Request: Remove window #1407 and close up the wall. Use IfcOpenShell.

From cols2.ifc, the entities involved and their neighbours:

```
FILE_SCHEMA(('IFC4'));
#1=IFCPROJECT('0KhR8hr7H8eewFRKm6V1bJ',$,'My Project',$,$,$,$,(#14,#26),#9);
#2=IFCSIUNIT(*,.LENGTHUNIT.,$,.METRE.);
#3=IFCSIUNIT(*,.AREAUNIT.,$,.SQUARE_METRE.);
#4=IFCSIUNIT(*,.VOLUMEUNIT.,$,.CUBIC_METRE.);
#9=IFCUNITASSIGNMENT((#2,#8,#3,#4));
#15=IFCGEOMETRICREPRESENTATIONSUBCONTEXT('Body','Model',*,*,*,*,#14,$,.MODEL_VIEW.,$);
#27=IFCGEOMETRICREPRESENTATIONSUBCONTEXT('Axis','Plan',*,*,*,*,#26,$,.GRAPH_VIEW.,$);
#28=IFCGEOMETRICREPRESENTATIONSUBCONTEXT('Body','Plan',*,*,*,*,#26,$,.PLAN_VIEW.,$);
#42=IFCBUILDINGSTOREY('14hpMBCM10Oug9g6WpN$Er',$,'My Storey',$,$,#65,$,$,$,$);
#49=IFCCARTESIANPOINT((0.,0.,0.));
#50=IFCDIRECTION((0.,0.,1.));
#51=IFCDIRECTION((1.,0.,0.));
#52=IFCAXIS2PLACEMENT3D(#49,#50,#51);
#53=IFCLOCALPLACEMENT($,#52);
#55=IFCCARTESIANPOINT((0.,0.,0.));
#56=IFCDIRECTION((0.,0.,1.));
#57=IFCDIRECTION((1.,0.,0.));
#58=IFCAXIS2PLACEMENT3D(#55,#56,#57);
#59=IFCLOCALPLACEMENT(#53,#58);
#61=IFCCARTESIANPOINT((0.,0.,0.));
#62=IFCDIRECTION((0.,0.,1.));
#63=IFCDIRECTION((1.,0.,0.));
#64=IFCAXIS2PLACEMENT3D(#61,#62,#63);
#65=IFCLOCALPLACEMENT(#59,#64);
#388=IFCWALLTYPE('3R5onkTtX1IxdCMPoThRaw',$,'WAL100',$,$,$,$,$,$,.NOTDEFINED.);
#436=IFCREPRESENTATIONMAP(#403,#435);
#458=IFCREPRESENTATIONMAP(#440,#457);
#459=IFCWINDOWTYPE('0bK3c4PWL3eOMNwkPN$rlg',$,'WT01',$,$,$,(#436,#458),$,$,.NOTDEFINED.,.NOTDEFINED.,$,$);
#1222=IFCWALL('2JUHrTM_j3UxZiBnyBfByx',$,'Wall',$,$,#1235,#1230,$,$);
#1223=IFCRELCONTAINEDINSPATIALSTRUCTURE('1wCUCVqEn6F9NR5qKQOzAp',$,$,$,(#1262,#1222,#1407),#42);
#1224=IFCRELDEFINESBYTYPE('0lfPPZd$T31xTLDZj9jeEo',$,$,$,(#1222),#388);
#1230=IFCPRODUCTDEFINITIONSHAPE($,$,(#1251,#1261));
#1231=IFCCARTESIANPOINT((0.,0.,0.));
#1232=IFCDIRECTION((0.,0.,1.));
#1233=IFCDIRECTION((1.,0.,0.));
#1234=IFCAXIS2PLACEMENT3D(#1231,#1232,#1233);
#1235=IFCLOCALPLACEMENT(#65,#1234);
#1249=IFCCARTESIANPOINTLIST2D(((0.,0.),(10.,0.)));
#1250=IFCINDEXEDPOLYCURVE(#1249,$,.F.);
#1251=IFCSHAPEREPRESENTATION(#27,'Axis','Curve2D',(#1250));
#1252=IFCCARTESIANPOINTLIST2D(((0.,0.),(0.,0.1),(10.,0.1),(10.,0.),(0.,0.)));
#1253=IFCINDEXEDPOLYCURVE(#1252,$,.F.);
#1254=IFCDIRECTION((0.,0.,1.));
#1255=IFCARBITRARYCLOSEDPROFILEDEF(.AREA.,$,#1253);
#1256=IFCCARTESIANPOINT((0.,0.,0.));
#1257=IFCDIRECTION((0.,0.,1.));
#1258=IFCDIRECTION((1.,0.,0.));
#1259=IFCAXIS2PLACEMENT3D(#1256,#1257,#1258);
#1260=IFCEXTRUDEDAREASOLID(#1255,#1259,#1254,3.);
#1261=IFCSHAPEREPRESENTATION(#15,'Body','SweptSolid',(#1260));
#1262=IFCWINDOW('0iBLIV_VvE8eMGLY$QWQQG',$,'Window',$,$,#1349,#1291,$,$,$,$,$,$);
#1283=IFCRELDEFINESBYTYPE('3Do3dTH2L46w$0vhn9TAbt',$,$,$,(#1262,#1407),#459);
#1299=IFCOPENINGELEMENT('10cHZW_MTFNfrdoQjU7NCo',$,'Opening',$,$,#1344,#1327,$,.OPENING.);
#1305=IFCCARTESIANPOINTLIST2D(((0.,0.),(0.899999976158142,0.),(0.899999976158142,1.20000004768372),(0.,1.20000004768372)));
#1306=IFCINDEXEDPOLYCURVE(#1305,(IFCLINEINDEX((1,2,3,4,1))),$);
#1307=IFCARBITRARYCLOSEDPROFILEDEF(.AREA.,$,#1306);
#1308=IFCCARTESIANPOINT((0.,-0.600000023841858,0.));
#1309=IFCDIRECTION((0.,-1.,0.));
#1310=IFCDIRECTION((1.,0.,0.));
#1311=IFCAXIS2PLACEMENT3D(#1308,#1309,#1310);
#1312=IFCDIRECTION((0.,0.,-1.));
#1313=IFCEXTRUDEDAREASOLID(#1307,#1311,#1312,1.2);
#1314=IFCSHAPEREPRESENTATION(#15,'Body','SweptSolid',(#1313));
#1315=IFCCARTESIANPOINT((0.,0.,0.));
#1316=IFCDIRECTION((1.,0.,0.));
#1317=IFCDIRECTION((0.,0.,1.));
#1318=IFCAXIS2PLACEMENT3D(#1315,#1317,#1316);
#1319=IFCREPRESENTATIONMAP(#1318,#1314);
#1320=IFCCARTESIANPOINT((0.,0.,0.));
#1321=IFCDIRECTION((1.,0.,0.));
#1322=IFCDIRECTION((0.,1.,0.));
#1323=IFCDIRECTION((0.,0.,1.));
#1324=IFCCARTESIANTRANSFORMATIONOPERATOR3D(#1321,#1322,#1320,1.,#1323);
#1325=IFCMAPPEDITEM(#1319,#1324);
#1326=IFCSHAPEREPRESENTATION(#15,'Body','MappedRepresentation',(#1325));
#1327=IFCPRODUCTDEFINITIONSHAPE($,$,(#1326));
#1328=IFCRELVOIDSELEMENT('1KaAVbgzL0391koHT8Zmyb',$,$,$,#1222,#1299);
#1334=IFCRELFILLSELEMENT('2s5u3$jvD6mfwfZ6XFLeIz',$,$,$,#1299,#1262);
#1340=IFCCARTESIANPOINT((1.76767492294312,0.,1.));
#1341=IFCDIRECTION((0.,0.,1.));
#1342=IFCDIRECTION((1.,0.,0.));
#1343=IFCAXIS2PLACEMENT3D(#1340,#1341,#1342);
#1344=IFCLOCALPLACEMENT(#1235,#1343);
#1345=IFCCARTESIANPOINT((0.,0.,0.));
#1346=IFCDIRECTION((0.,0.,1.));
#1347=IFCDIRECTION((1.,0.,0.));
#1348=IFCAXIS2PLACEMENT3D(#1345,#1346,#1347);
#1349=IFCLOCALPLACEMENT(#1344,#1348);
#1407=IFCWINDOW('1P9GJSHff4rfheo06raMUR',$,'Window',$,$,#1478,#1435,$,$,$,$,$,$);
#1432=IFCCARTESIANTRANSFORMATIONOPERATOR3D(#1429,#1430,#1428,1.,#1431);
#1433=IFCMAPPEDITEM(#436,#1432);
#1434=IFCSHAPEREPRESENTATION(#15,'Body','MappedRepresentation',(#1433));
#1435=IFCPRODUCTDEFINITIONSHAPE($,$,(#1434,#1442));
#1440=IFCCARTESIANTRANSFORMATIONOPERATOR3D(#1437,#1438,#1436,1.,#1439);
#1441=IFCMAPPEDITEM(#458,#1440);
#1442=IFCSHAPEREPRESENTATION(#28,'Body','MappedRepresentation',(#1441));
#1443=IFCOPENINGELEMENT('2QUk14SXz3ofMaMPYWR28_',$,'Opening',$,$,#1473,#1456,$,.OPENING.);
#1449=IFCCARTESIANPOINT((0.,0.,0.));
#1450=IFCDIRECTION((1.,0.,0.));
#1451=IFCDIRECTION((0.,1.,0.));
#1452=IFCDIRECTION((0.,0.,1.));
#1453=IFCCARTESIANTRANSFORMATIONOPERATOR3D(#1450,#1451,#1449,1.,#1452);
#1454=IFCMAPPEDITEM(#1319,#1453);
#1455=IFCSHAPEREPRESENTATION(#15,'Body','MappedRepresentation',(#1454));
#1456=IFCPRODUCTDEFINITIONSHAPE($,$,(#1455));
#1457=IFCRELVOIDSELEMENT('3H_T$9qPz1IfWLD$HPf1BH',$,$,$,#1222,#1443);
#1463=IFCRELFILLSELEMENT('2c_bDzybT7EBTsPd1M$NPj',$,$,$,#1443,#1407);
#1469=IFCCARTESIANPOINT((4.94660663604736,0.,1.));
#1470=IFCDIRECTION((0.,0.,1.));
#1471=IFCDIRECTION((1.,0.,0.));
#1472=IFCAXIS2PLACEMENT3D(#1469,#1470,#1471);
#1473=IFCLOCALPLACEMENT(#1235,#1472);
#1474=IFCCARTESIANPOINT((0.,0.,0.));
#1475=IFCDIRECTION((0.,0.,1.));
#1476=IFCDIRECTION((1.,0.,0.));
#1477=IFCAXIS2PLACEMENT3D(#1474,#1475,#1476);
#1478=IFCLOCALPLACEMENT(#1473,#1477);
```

```python
import ifcopenshell
import ifcopenshell.api.feature
import ifcopenshell.api.root
import ifcopenshell.geom
import ifcopenshell.util.shape

model = ifcopenshell.open("cols2.ifc")
settings = ifcopenshell.geom.settings()


def volume(element):
    """Net volume in cubic metres, openings subtracted."""
    shape = ifcopenshell.geom.create_shape(settings, element)
    return ifcopenshell.util.shape.get_volume(shape.geometry)


window = model.by_guid("1P9GJSHff4rfheo06raMUR")
opening = window.FillsVoids[0].RelatingOpeningElement
wall = opening.VoidsElements[0].RelatingBuildingElement
before = volume(wall)

ifcopenshell.api.root.remove_product(model, product=window)
ifcopenshell.api.feature.remove_feature(model, feature=opening)

after = volume(wall)

print(f"wall volume {before:.3f} -> {after:.3f} m3")

model.write("cols2_updated.ifc")
```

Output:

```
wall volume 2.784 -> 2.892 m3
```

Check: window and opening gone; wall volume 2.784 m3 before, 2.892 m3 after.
